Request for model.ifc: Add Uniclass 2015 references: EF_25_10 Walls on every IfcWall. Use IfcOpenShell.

First a look at what the model holds.

```python
import ifcopenshell

model = ifcopenshell.open("model.ifc")
print(model.schema)
print("classifications:", [c.Name for c in model.by_type("IfcClassification")])
for ifc_class in ("IfcDoor", "IfcRoof", "IfcStair", "IfcWall", "IfcWindow"):
    print(ifc_class, len(model.by_type(ifc_class)))
```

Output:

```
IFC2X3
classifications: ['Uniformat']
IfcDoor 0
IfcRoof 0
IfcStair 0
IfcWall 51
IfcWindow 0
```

```python
import ifcopenshell
import ifcopenshell.api.classification

model = ifcopenshell.open("model.ifc")

# IFC2X3 requires Source and Edition and has no link from the project to the system.
system = model.create_entity("IfcClassification", Source="NBS", Edition="2015", Name="Uniclass 2015")

codes = {
    "IfcWall": ("EF_25_10", "Walls"),
}
for ifc_class, (code, name) in codes.items():
    products = model.by_type(ifc_class)
    ifcopenshell.api.classification.add_reference(
        model, products=products, classification=system, identification=code, name=name
    )
    print(code, len(products))

model.write("model_rev.ifc")
```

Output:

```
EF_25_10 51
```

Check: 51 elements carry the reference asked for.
